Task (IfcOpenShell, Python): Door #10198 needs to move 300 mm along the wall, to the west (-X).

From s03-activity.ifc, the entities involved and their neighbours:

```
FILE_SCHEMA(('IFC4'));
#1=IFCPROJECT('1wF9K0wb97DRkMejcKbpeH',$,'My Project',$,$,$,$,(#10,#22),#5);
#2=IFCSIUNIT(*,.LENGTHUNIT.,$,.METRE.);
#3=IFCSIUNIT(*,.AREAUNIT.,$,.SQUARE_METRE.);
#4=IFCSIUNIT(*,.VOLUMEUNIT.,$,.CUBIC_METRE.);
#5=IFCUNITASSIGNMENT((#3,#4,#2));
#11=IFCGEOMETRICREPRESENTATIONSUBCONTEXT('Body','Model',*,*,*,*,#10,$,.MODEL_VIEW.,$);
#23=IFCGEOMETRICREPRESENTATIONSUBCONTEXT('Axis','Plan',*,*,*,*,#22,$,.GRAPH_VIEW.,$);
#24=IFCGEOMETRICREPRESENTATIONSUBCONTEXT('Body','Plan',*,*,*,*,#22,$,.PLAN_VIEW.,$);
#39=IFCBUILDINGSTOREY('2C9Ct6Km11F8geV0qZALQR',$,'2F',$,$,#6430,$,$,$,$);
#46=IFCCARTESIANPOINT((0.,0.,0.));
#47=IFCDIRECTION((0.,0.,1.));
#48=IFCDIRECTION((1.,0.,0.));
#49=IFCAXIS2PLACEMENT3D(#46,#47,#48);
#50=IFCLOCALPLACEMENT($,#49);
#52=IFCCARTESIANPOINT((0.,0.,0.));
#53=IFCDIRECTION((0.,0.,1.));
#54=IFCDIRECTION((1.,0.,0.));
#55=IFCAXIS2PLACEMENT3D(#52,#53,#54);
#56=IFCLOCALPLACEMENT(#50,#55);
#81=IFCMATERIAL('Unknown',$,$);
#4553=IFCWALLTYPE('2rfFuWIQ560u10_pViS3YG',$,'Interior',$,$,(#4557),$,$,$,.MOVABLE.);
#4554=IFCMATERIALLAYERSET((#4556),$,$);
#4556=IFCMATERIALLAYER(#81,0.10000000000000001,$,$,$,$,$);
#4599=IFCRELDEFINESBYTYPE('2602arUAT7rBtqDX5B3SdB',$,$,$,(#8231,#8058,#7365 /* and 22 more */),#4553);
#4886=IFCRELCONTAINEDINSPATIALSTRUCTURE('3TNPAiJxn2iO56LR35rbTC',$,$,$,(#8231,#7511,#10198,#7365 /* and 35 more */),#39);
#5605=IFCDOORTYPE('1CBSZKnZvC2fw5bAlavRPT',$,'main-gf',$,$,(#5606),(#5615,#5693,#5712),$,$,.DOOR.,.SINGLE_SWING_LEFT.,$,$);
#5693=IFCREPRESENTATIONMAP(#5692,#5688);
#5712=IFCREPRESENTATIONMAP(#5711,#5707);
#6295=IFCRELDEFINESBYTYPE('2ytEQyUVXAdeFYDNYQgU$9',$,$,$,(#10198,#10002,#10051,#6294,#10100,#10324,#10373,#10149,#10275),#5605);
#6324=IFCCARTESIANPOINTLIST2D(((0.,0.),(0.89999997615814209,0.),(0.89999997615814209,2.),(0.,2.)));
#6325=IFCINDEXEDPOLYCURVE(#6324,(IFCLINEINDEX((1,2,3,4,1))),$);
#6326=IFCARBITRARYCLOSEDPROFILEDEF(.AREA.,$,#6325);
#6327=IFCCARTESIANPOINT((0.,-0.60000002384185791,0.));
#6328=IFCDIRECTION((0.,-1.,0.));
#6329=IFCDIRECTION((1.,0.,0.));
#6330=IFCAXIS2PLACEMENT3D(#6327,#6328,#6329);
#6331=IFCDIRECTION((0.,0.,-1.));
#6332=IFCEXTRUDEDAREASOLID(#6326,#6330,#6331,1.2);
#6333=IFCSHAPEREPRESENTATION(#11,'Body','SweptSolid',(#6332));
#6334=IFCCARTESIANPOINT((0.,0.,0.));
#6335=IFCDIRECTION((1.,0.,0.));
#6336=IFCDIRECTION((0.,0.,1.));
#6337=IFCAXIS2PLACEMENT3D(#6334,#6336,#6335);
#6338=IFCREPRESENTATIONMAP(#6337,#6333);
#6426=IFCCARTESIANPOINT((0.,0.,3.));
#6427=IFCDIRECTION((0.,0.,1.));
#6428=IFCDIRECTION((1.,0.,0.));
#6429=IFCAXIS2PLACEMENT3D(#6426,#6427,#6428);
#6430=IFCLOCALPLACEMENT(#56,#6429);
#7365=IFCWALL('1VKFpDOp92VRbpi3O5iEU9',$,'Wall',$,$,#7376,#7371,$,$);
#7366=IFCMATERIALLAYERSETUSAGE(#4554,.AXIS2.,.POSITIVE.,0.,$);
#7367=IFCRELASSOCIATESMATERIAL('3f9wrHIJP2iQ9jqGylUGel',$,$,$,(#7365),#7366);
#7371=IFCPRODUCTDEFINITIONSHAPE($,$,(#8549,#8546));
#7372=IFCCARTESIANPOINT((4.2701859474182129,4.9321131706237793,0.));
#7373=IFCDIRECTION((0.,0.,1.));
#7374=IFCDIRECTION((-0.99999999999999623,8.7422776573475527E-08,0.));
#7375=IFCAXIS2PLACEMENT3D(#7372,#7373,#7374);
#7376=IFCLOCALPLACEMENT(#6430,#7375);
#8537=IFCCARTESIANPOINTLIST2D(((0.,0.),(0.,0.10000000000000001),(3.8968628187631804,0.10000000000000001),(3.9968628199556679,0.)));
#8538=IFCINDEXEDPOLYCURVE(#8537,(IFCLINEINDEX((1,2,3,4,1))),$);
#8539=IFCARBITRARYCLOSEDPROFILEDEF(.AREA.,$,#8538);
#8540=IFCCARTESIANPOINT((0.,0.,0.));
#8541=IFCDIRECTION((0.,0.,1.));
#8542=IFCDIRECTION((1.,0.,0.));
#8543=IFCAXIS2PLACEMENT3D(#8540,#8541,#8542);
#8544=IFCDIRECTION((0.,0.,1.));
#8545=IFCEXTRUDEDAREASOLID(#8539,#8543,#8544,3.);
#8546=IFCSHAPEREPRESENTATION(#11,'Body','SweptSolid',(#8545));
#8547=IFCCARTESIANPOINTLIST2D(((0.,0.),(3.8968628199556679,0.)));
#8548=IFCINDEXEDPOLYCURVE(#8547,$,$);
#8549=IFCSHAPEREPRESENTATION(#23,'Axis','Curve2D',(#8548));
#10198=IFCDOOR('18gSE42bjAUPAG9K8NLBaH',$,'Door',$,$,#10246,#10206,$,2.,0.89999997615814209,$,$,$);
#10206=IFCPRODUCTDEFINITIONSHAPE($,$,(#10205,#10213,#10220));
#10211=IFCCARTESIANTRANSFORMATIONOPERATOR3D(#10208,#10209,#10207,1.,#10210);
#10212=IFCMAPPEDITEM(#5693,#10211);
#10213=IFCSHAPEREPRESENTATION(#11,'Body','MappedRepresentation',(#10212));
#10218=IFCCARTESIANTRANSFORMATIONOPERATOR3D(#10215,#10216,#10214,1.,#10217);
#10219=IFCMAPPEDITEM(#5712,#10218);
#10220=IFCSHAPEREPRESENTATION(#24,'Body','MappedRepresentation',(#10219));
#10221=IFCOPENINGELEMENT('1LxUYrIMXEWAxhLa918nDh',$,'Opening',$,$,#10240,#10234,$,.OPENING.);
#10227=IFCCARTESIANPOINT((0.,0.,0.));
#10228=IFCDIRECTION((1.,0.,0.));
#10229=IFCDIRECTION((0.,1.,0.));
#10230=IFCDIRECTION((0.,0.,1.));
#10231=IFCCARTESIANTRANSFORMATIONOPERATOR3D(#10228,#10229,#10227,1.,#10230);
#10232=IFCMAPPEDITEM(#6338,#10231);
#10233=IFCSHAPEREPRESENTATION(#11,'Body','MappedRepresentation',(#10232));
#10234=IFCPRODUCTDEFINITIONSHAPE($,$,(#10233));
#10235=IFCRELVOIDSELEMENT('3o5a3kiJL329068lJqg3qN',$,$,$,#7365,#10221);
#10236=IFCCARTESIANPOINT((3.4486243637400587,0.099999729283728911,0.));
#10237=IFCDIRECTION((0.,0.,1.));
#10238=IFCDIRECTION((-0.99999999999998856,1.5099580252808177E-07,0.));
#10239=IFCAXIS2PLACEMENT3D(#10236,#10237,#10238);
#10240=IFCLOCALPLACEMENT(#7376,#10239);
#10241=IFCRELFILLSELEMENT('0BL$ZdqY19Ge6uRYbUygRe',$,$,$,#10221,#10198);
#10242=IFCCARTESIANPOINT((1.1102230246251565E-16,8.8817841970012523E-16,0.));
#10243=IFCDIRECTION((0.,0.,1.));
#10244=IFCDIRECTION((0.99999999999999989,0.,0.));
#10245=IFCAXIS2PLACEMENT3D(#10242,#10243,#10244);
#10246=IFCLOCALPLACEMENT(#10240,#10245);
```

```python
import ifcopenshell
import ifcopenshell.api.geometry
import ifcopenshell.util.placement
import ifcopenshell.util.unit

model = ifcopenshell.open("s03-activity.ifc")
unit_scale = ifcopenshell.util.unit.calculate_unit_scale(model)

door = model.by_guid("18gSE42bjAUPAG9K8NLBaH")
opening = door.FillsVoids[0].RelatingOpeningElement
wall = opening.VoidsElements[0].RelatingBuildingElement

wall_matrix = ifcopenshell.util.placement.get_local_placement(wall.ObjectPlacement)
shift = wall_matrix[:3, 0] * 0.3 / unit_scale
before = ifcopenshell.util.placement.get_local_placement(door.ObjectPlacement)[:3, 3].copy()

# The door is placed relative to its opening, so it follows when the opening moves.
matrix = ifcopenshell.util.placement.get_local_placement(opening.ObjectPlacement)
matrix[:3, 3] += shift
ifcopenshell.api.geometry.edit_object_placement(
    model, product=opening, matrix=matrix, is_si=False, should_transform_children=True
)

after = ifcopenshell.util.placement.get_local_placement(door.ObjectPlacement)[:3, 3]
print("door moved by", (after - before).round(3) + 0.0)

model.write("s03-activity_edited.ifc")
```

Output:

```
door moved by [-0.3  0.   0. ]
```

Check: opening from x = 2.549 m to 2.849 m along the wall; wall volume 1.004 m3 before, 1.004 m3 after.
